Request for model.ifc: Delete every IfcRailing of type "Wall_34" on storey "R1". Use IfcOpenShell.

First a look at what the model holds.

```python
import ifcopenshell
import ifcopenshell.util.element

model = ifcopenshell.open("model.ifc")
print(model.schema)
storey = next(s for s in model.by_type("IfcBuildingStorey") if s.Name == "R1")
railings = [e for e in ifcopenshell.util.element.get_decomposition(storey) if e.is_a("IfcRailing")]
seen = {}
for e in railings:
    element_type = ifcopenshell.util.element.get_type(e)
    name = element_type.Name if element_type not in (None, e) else None
    seen[name] = seen.get(name, 0) + 1
for name, count in sorted(seen.items(), key=str):
    print(count, "x", name)
```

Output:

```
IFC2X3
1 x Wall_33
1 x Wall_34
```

```python
import ifcopenshell
import ifcopenshell.api.root
import ifcopenshell.util.element

model = ifcopenshell.open("model.ifc")

storey = next(s for s in model.by_type("IfcBuildingStorey") if s.Name == "R1")
railings = [e for e in ifcopenshell.util.element.get_decomposition(storey) if e.is_a("IfcRailing")]
targets = [e for e in railings if (t := ifcopenshell.util.element.get_type(e)) not in (None, e) and t.Name == "Wall_34"]

for e in targets:
    ifcopenshell.api.root.remove_product(model, product=e)
print(len(targets), "removed")

model.write("model_v2.ifc")
```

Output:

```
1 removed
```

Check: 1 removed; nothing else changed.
